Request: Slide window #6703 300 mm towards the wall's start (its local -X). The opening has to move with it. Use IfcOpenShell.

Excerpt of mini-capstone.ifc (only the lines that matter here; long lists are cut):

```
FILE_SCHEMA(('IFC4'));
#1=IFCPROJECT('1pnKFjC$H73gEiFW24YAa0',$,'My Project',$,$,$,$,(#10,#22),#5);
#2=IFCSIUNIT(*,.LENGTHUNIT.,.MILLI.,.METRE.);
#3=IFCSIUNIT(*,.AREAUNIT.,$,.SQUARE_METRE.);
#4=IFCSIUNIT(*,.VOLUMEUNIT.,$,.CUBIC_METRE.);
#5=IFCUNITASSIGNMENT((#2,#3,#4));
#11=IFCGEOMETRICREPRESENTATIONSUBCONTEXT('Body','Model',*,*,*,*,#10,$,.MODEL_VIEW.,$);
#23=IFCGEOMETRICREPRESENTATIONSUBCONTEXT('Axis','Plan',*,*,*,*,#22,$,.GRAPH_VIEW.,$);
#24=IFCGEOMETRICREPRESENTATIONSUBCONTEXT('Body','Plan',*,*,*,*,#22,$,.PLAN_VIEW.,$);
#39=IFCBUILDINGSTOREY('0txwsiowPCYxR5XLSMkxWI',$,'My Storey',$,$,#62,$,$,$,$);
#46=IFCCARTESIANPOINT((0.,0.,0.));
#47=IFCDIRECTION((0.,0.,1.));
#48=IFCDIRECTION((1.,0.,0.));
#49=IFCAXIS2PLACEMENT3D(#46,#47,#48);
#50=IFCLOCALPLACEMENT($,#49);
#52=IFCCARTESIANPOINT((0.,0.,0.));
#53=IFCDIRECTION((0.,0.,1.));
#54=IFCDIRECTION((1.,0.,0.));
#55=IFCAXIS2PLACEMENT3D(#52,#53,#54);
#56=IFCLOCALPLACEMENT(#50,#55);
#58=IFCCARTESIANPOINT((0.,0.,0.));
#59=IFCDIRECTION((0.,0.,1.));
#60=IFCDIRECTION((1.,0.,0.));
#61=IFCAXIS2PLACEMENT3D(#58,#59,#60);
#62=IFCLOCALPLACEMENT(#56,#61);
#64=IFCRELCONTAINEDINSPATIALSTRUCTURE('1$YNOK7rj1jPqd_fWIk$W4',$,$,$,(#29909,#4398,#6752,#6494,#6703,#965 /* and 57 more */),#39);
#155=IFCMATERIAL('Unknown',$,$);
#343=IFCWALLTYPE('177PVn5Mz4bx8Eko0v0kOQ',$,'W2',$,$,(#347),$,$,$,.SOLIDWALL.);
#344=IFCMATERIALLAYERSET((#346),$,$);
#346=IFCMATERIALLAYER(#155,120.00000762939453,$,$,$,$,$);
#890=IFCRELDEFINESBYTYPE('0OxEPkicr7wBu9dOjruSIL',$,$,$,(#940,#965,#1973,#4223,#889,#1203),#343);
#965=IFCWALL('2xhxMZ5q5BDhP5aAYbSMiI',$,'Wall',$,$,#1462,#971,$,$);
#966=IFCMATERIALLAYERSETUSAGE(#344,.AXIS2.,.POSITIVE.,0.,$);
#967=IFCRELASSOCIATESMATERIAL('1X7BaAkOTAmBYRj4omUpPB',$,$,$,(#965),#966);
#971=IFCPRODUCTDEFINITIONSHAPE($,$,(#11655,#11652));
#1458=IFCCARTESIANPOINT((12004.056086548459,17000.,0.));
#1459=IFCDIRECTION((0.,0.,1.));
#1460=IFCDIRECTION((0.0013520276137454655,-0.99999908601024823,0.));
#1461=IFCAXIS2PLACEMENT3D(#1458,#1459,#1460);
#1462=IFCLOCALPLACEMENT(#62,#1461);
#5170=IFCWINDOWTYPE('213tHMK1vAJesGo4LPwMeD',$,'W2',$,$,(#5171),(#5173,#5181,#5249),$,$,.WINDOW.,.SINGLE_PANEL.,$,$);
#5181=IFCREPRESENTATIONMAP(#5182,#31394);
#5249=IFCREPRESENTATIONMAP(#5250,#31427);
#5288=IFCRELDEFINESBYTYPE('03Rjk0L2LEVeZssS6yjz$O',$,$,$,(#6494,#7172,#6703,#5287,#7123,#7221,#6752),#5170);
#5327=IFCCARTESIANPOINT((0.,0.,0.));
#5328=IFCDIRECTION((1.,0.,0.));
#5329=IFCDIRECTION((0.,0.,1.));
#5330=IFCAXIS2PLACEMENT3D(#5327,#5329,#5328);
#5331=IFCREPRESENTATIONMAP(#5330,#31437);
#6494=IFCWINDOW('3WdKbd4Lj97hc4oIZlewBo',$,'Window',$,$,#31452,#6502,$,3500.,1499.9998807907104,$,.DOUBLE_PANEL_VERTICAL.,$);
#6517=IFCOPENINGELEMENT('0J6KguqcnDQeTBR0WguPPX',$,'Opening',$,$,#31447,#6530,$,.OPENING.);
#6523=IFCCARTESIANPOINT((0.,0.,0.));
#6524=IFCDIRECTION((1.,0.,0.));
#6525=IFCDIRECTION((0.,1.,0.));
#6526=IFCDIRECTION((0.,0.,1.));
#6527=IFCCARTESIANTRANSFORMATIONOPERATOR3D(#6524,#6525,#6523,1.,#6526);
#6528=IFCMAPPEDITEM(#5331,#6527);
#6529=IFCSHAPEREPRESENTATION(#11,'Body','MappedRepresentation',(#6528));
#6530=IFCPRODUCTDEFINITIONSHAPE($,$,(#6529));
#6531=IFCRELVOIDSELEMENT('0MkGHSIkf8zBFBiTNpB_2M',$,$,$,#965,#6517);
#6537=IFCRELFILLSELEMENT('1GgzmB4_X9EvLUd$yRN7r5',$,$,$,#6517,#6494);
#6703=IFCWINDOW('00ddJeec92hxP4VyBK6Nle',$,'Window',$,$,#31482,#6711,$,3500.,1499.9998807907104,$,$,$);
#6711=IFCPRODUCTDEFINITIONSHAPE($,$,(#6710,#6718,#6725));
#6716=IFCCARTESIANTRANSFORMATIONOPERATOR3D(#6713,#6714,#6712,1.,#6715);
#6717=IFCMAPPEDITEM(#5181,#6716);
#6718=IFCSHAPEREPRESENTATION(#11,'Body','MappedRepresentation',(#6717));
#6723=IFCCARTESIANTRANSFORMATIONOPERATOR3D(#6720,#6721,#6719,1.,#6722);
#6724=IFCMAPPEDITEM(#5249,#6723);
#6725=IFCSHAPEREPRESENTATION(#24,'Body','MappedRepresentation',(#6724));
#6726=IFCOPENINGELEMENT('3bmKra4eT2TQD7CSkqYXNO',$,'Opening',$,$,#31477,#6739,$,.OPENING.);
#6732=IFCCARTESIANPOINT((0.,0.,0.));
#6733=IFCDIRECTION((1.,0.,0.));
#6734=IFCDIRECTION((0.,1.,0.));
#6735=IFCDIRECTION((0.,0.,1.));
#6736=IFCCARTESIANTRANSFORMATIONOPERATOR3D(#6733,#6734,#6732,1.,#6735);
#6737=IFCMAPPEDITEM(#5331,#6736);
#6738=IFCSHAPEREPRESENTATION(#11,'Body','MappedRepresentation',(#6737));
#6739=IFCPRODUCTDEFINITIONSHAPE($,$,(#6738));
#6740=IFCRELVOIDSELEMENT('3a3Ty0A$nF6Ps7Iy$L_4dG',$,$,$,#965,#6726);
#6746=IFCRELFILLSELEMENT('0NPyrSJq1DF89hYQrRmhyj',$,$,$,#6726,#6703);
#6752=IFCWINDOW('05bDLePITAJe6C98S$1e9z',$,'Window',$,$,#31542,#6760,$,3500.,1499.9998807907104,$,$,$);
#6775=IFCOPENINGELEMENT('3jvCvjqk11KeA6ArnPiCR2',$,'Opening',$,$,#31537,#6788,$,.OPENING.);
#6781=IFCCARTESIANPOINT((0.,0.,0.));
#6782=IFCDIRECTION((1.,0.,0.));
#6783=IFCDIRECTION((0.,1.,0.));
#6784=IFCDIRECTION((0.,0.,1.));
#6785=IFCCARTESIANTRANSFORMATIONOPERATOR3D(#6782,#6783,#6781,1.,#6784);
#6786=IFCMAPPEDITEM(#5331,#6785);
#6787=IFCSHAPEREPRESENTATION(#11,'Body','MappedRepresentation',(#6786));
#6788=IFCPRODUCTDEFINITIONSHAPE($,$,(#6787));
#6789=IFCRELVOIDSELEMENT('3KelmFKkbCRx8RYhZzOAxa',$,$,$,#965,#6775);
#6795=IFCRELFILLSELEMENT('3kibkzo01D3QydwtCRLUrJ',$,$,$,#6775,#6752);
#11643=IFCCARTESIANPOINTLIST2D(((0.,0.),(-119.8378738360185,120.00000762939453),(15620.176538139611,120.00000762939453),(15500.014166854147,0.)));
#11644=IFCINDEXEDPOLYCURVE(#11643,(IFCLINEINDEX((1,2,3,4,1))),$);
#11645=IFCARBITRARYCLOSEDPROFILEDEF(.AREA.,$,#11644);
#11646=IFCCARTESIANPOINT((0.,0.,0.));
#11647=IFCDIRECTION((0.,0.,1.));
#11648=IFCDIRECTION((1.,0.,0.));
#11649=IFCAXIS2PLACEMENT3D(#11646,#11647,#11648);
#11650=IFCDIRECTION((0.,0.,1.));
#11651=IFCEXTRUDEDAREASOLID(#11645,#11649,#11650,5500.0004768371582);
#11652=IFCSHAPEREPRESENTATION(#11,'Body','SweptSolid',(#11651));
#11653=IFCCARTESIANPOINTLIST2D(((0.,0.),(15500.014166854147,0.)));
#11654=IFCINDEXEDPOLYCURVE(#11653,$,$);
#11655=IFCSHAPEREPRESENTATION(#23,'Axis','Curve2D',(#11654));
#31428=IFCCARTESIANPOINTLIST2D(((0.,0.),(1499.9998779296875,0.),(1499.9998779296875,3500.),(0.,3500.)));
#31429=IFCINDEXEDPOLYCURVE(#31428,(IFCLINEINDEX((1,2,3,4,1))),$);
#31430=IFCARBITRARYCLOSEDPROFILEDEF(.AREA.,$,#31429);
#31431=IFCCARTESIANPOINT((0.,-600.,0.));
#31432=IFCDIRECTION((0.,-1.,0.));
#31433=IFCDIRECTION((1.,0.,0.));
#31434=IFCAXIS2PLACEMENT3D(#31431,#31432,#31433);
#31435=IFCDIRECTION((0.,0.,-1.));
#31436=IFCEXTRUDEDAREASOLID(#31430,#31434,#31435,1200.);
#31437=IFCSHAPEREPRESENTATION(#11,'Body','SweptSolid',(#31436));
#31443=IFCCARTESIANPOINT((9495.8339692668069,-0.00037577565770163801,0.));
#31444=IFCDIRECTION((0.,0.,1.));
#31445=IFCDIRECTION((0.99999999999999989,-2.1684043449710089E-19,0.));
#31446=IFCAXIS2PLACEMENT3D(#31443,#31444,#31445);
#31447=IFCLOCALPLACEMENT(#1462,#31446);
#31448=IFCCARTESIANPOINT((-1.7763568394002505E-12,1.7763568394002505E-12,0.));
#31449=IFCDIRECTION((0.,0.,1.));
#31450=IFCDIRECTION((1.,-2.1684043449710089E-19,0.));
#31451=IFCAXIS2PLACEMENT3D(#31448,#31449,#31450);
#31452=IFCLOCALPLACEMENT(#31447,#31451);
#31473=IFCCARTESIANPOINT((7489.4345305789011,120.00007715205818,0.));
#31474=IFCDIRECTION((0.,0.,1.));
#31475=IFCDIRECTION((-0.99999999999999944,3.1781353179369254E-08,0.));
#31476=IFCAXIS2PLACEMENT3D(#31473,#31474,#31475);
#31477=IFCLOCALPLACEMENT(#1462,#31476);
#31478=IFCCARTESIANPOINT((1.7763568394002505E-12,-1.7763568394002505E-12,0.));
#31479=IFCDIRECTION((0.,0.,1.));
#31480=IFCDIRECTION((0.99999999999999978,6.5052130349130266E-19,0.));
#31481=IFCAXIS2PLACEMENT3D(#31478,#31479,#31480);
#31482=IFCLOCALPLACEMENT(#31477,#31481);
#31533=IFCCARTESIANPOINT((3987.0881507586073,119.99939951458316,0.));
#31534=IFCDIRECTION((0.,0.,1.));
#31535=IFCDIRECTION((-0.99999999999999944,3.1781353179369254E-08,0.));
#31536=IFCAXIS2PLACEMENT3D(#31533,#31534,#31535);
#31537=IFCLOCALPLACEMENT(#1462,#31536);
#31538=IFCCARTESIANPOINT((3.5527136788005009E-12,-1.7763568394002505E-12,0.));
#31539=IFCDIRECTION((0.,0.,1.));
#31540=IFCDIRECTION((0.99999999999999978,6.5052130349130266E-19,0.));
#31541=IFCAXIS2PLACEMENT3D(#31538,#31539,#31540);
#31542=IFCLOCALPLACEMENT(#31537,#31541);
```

```python
import ifcopenshell
import ifcopenshell.api.geometry
import ifcopenshell.util.placement
import ifcopenshell.util.unit

model = ifcopenshell.open("mini-capstone.ifc")
unit_scale = ifcopenshell.util.unit.calculate_unit_scale(model)

window = model.by_id(6703)
opening = window.FillsVoids[0].RelatingOpeningElement
wall = opening.VoidsElements[0].RelatingBuildingElement

wall_matrix = ifcopenshell.util.placement.get_local_placement(wall.ObjectPlacement)
shift = wall_matrix[:3, 0] * -0.3 / unit_scale
before = ifcopenshell.util.placement.get_local_placement(window.ObjectPlacement)[:3, 3].copy()

# The window is placed relative to its opening, so it follows when the opening moves.
matrix = ifcopenshell.util.placement.get_local_placement(opening.ObjectPlacement)
matrix[:3, 3] += shift
ifcopenshell.api.geometry.edit_object_placement(
    model, product=opening, matrix=matrix, is_si=False, should_transform_children=True
)

after = ifcopenshell.util.placement.get_local_placement(window.ObjectPlacement)[:3, 3]
print("window moved by", (after - before).round(3) + 0.0)

model.write("mini-capstone-out.ifc")
```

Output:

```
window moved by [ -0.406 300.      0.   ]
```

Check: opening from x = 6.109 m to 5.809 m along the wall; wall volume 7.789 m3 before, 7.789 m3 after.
